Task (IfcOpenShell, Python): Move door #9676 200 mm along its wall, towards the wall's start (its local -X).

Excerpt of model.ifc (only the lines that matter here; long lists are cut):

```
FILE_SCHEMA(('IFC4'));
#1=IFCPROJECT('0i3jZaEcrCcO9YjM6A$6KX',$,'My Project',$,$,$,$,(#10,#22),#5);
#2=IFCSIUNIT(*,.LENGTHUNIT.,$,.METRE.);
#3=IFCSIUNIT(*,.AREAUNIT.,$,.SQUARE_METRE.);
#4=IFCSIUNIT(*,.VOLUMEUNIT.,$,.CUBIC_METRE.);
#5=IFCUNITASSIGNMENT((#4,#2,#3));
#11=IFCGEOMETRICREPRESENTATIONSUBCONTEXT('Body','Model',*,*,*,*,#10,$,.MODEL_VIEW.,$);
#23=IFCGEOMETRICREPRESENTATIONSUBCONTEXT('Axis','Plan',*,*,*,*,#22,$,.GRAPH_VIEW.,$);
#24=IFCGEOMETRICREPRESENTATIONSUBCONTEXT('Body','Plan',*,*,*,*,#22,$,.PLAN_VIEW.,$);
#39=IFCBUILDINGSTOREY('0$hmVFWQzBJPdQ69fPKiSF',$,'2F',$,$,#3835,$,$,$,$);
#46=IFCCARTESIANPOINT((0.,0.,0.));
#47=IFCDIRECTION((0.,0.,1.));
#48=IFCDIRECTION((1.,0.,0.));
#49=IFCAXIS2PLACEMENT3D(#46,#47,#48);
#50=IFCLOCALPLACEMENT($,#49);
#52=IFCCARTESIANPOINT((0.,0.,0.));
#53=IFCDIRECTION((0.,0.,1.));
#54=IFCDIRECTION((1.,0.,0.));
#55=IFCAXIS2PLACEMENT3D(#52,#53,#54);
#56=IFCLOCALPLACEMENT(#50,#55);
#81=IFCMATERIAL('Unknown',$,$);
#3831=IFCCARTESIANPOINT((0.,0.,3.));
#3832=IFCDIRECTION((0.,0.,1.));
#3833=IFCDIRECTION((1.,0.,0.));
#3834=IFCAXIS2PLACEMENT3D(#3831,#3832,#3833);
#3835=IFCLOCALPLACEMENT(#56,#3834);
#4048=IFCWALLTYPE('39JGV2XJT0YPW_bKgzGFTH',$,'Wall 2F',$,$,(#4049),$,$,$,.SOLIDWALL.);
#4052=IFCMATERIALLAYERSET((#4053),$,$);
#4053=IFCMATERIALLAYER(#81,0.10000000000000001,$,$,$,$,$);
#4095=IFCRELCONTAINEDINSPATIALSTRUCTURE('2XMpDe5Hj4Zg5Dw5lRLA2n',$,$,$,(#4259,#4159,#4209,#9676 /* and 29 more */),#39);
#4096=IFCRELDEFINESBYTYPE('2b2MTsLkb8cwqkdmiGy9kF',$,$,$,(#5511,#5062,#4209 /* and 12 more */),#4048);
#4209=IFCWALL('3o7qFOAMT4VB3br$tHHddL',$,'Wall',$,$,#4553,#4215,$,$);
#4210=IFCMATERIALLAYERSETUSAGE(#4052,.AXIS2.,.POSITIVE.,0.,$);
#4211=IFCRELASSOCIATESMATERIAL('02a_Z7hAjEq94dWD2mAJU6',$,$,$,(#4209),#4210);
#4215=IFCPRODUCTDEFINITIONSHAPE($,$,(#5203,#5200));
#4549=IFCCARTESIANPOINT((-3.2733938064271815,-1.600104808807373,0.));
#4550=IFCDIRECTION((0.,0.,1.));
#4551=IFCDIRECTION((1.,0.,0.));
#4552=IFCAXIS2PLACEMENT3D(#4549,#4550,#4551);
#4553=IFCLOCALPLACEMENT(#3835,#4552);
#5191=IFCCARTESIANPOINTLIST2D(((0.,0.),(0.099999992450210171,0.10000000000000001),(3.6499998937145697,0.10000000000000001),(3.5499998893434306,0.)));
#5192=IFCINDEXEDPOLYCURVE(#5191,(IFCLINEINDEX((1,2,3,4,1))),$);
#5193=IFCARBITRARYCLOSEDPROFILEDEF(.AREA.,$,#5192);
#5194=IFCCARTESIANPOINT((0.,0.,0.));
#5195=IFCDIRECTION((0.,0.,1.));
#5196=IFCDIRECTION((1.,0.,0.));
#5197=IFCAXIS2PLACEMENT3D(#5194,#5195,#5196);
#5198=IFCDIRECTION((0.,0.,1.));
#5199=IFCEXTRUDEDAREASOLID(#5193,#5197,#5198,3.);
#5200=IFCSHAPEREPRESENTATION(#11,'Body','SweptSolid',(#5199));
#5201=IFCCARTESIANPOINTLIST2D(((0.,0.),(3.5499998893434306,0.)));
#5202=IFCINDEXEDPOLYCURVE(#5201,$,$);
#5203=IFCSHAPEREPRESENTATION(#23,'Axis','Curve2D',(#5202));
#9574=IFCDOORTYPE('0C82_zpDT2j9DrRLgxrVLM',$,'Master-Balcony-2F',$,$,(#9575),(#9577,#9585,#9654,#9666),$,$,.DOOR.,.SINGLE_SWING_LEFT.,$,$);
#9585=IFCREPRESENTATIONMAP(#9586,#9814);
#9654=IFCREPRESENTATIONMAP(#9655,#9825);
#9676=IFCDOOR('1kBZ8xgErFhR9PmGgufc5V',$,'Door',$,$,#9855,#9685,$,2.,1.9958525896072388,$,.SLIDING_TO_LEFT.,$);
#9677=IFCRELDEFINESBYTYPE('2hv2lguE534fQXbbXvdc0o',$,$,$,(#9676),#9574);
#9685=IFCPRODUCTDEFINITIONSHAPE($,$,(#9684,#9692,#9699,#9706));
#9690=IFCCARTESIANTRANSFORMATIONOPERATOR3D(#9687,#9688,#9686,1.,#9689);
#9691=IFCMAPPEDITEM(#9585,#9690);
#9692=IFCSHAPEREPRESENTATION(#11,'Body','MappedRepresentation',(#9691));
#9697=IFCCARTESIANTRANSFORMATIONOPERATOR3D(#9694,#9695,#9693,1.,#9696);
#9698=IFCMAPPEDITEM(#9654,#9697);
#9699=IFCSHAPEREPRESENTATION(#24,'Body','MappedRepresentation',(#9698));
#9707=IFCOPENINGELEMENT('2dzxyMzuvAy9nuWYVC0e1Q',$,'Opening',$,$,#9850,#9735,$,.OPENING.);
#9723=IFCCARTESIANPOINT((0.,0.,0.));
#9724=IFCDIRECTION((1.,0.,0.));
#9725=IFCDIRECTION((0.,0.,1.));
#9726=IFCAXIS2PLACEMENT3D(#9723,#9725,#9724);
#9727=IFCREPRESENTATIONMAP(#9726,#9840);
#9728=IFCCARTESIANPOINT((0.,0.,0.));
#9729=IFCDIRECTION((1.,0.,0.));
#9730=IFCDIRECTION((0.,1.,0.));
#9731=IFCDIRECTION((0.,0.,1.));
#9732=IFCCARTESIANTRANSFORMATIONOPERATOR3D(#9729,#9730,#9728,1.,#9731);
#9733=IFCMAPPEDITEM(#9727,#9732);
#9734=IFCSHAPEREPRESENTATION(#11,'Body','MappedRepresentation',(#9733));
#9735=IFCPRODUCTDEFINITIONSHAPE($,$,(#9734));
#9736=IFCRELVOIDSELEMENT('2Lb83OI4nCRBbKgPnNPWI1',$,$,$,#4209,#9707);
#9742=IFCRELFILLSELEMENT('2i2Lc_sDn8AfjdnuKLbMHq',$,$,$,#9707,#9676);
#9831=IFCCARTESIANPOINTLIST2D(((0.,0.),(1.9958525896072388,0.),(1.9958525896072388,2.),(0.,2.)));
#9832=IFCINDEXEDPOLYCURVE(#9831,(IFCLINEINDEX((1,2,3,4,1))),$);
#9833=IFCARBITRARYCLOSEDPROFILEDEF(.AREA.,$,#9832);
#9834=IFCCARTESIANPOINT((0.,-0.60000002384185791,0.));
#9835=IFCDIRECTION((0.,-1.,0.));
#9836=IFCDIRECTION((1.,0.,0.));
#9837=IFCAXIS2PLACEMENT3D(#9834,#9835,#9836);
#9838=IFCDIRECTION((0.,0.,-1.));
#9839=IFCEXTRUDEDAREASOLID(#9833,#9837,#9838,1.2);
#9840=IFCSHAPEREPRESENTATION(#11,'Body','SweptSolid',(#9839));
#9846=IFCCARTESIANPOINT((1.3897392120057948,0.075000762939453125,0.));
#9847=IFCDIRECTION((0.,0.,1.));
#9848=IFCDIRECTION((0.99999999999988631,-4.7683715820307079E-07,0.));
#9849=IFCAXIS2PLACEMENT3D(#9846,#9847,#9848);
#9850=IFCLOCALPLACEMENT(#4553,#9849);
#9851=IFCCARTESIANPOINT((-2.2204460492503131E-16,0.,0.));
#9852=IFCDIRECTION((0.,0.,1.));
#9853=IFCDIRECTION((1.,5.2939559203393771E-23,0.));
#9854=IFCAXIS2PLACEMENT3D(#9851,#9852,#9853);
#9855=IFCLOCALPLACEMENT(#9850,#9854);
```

```python
import ifcopenshell
import ifcopenshell.api.geometry
import ifcopenshell.util.placement

model = ifcopenshell.open("model.ifc")

door = model.by_guid("1kBZ8xgErFhR9PmGgufc5V")
opening = door.FillsVoids[0].RelatingOpeningElement
wall = opening.VoidsElements[0].RelatingBuildingElement

wall_matrix = ifcopenshell.util.placement.get_local_placement(wall.ObjectPlacement)
shift = wall_matrix[:3, 0] * -0.2
before = ifcopenshell.util.placement.get_local_placement(door.ObjectPlacement)[:3, 3].copy()

# The door is placed relative to its opening, so it follows when the opening moves.
matrix = ifcopenshell.util.placement.get_local_placement(opening.ObjectPlacement)
matrix[:3, 3] += shift
ifcopenshell.api.geometry.edit_object_placement(
    model, product=opening, matrix=matrix, is_si=False, should_transform_children=True
)

after = ifcopenshell.util.placement.get_local_placement(door.ObjectPlacement)[:3, 3]
print("door moved by", (after - before).round(3) + 0.0)

model.write("model_rev.ifc")
```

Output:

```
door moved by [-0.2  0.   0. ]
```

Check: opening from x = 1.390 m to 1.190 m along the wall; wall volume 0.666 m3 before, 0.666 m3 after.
